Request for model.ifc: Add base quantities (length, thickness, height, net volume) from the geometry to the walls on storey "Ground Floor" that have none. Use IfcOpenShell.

First a look at what the model holds.

```python
import ifcopenshell
import ifcopenshell.util.element
import ifcopenshell.util.unit

model = ifcopenshell.open("model.ifc")
print(model.schema)
for unit_type in ("LENGTHUNIT", "AREAUNIT", "VOLUMEUNIT"):
    print(unit_type, ifcopenshell.util.unit.calculate_unit_scale(model, unit_type))
storey = next(s for s in model.by_type("IfcBuildingStorey") if s.Name == "Ground Floor")
walls = [e for e in ifcopenshell.util.element.get_decomposition(storey) if e.is_a("IfcWall")]
for e in sorted(walls, key=lambda e: e.id()):
    print(e.id(), e.is_a(), e.Name, list(ifcopenshell.util.element.get_psets(e, qtos_only=True)), sep=" | ")
```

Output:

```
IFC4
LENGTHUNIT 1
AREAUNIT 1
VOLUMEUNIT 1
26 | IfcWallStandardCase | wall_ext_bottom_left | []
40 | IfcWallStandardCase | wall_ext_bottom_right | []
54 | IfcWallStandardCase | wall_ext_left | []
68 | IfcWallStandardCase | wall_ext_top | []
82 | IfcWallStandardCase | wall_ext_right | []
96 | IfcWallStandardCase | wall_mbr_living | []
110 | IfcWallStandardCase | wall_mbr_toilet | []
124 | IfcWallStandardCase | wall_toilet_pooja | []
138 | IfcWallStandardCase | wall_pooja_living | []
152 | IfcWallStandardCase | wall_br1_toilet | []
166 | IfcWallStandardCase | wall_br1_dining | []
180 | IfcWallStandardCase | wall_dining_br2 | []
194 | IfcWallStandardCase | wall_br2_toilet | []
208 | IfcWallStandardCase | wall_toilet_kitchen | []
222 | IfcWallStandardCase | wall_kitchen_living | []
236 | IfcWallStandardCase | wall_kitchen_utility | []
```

```python
import ifcopenshell
import ifcopenshell.api.pset
import ifcopenshell.geom
import ifcopenshell.util.element
import ifcopenshell.util.shape
import ifcopenshell.util.unit

model = ifcopenshell.open("model.ifc")
unit_scale = ifcopenshell.util.unit.calculate_unit_scale(model)
volume_scale = ifcopenshell.util.unit.calculate_unit_scale(model, "VOLUMEUNIT")
settings = ifcopenshell.geom.settings()

storey = next(s for s in model.by_type("IfcBuildingStorey") if s.Name == "Ground Floor")
walls = [e for e in ifcopenshell.util.element.get_decomposition(storey) if e.is_a("IfcWall")]

for e in sorted(walls, key=lambda e: e.id()):
    if ifcopenshell.util.element.get_psets(e, qtos_only=True, should_inherit=False):
        continue
    # Geometry comes back in metres, in the element's own axes.
    shape = ifcopenshell.geom.create_shape(settings, e)
    values = {
        "Length": ifcopenshell.util.shape.get_x(shape.geometry) / unit_scale,
        "Width": ifcopenshell.util.shape.get_y(shape.geometry) / unit_scale,
        "Height": ifcopenshell.util.shape.get_z(shape.geometry) / unit_scale,
        "NetVolume": ifcopenshell.util.shape.get_volume(shape.geometry) / volume_scale,
    }
    qto = ifcopenshell.api.pset.add_qto(model, product=e, name="Qto_WallBaseQuantities")
    ifcopenshell.api.pset.edit_qto(model, qto=qto, properties=values)
    print(e.id(), {k: round(v, 3) for k, v in values.items()})

model.write("model_updated.ifc")
```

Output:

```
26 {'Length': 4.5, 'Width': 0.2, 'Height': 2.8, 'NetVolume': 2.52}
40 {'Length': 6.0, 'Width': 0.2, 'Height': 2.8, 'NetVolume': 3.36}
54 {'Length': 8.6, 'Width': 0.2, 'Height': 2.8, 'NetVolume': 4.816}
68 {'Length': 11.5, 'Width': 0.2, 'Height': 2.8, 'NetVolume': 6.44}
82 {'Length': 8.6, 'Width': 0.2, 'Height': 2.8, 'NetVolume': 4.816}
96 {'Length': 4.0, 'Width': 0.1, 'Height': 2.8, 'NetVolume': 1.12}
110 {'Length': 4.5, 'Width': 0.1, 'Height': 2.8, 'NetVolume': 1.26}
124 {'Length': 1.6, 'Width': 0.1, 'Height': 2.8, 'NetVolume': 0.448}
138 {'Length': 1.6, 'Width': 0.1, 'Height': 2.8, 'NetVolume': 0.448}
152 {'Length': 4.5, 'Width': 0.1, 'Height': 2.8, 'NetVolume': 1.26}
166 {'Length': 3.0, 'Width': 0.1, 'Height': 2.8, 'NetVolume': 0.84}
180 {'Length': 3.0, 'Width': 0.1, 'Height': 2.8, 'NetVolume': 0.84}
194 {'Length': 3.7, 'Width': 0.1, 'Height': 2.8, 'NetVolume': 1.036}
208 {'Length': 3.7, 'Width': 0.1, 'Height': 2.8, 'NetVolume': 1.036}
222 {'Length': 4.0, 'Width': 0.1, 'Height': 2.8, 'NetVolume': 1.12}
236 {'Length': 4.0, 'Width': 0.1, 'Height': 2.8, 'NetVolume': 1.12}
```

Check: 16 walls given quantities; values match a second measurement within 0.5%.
